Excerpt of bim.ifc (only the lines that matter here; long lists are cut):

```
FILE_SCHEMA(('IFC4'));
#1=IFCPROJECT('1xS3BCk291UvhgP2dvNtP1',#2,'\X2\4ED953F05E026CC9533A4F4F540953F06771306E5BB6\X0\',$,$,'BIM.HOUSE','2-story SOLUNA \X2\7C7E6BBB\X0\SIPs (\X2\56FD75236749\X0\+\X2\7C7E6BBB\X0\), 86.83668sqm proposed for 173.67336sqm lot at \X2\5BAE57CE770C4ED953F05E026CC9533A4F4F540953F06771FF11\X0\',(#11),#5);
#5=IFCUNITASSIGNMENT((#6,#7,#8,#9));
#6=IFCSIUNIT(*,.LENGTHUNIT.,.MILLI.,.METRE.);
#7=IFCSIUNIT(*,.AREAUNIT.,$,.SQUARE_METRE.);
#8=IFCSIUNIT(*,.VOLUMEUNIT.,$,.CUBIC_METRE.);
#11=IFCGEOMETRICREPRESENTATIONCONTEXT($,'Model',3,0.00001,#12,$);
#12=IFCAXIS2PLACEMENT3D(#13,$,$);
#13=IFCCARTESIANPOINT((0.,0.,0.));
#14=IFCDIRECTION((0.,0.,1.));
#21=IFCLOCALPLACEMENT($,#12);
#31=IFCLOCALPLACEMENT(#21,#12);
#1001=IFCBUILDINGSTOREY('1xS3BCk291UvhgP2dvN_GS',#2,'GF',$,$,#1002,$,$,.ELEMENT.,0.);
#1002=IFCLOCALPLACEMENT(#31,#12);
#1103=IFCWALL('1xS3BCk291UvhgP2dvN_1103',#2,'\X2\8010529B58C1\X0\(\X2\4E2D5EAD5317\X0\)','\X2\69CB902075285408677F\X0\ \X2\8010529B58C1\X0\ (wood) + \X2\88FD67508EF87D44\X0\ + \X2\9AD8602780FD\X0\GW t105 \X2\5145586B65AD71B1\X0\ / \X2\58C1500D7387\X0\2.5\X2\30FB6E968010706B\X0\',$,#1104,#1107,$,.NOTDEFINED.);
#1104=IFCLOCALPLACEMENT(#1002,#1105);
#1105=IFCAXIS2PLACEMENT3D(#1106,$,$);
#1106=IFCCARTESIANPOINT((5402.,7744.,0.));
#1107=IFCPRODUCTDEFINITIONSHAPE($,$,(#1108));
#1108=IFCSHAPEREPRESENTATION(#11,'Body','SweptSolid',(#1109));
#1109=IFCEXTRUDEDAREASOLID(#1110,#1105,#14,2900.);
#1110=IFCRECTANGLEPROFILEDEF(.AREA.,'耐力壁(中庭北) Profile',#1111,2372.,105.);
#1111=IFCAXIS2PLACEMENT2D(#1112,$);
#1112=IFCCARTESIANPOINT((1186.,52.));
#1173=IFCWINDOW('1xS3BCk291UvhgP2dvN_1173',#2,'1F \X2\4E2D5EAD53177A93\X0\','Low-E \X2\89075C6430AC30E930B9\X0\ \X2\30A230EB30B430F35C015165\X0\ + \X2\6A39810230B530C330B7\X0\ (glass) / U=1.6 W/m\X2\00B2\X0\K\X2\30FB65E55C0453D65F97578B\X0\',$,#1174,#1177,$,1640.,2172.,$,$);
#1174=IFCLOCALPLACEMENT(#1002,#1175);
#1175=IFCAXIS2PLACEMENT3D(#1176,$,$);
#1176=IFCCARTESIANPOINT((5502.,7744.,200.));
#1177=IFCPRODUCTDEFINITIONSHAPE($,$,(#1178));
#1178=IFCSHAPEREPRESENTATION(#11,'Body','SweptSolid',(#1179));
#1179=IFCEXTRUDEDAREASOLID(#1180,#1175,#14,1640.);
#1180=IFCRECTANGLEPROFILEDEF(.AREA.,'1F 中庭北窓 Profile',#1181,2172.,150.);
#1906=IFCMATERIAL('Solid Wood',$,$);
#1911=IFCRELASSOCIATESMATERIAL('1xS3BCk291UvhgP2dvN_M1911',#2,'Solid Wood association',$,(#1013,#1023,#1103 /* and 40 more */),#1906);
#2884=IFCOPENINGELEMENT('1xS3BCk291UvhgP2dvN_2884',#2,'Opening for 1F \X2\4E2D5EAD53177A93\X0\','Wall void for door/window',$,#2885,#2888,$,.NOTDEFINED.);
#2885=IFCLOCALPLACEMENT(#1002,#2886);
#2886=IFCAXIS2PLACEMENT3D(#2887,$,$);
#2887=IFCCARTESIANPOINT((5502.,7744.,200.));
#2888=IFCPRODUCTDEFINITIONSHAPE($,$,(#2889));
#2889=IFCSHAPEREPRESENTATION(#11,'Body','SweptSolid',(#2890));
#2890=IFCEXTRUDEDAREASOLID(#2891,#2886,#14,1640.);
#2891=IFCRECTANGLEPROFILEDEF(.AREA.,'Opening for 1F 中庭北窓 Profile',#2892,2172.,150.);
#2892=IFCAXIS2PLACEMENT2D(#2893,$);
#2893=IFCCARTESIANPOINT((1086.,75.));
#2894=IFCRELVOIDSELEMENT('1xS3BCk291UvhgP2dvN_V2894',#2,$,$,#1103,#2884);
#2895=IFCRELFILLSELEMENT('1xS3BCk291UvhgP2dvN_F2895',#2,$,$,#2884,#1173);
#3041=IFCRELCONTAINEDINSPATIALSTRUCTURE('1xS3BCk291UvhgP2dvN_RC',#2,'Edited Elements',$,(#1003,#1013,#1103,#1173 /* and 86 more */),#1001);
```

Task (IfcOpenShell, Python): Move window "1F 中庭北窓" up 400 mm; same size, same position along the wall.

```python
import numpy as np
import ifcopenshell
import ifcopenshell.api.geometry
import ifcopenshell.util.placement
import ifcopenshell.util.unit

model = ifcopenshell.open("bim.ifc")
unit_scale = ifcopenshell.util.unit.calculate_unit_scale(model)

window = model.by_guid("1xS3BCk291UvhgP2dvN_1173")
opening = window.FillsVoids[0].RelatingOpeningElement
dz = 400.0

shift = np.array([0.0, 0.0, dz])
# The window is not placed relative to its opening, so move both.
for product in (opening, window):
    matrix = ifcopenshell.util.placement.get_local_placement(product.ObjectPlacement)
    matrix[:3, 3] += shift
    ifcopenshell.api.geometry.edit_object_placement(model, product=product, matrix=matrix, is_si=False)

print(f"moved by {dz * unit_scale:+.3f} m")

model.write("bim-out.ifc")
```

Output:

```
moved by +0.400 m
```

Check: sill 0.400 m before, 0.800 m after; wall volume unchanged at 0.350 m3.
